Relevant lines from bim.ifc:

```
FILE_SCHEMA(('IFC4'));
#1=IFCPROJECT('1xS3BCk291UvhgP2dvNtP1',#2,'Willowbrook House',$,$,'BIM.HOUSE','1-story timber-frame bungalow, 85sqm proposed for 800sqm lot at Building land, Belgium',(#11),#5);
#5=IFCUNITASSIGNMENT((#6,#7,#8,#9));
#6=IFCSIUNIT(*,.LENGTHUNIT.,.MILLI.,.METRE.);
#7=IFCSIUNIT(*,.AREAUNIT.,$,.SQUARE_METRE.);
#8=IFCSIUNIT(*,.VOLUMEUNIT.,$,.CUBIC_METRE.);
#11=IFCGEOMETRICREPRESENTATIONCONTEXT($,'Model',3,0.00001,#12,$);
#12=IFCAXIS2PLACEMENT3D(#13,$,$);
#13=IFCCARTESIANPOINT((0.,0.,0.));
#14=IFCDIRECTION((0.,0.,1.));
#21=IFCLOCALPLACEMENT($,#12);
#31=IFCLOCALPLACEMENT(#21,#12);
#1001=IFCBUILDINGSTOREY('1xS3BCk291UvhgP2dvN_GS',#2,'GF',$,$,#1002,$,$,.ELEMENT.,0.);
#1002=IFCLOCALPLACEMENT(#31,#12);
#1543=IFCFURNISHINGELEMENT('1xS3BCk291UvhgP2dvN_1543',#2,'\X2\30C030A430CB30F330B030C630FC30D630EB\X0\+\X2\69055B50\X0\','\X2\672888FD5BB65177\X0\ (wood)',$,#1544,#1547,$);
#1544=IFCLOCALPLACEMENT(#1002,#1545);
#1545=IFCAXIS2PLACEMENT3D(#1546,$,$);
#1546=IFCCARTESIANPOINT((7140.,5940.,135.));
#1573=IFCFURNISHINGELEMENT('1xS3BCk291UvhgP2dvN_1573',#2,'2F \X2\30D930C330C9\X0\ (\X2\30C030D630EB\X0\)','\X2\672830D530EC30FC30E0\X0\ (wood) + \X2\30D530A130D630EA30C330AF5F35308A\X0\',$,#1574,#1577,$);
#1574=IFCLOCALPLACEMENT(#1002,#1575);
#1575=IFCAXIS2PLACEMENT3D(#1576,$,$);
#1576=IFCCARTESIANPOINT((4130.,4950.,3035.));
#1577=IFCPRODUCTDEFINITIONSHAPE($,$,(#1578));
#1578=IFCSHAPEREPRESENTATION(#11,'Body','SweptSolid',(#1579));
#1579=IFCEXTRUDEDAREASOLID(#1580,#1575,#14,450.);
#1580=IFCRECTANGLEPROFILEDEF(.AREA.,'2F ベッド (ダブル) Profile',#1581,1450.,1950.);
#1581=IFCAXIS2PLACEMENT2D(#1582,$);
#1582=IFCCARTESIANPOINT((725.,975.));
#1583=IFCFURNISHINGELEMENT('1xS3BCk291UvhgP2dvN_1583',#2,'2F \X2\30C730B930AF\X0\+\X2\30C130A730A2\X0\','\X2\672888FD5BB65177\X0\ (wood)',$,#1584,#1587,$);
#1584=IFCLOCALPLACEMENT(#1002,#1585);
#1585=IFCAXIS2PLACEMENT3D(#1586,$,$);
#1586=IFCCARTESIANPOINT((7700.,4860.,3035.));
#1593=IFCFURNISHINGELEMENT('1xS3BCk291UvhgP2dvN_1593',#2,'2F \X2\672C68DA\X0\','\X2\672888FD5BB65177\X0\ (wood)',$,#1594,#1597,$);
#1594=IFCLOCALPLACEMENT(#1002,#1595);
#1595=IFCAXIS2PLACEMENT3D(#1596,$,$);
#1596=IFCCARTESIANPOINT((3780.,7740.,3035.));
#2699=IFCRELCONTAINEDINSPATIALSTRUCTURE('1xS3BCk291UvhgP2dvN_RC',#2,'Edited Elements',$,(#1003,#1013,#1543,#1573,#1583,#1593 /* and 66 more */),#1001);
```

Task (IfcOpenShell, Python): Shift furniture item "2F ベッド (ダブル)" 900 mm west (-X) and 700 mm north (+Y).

```python
import ifcopenshell
import ifcopenshell.api.geometry
import ifcopenshell.util.placement

model = ifcopenshell.open("bim.ifc")

item = model.by_guid("1xS3BCk291UvhgP2dvN_1573")
matrix = ifcopenshell.util.placement.get_local_placement(item.ObjectPlacement)
matrix[0, 3] -= 900.0
matrix[1, 3] += 700.0
ifcopenshell.api.geometry.edit_object_placement(model, product=item, matrix=matrix, is_si=False)

print(ifcopenshell.util.placement.get_local_placement(item.ObjectPlacement).round(3) + 0.0)

model.write("bim_updated.ifc")
```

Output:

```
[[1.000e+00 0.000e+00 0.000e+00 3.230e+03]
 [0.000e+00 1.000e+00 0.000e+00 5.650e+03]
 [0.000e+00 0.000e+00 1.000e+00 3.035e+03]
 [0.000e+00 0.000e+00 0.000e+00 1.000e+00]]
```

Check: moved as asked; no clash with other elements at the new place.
